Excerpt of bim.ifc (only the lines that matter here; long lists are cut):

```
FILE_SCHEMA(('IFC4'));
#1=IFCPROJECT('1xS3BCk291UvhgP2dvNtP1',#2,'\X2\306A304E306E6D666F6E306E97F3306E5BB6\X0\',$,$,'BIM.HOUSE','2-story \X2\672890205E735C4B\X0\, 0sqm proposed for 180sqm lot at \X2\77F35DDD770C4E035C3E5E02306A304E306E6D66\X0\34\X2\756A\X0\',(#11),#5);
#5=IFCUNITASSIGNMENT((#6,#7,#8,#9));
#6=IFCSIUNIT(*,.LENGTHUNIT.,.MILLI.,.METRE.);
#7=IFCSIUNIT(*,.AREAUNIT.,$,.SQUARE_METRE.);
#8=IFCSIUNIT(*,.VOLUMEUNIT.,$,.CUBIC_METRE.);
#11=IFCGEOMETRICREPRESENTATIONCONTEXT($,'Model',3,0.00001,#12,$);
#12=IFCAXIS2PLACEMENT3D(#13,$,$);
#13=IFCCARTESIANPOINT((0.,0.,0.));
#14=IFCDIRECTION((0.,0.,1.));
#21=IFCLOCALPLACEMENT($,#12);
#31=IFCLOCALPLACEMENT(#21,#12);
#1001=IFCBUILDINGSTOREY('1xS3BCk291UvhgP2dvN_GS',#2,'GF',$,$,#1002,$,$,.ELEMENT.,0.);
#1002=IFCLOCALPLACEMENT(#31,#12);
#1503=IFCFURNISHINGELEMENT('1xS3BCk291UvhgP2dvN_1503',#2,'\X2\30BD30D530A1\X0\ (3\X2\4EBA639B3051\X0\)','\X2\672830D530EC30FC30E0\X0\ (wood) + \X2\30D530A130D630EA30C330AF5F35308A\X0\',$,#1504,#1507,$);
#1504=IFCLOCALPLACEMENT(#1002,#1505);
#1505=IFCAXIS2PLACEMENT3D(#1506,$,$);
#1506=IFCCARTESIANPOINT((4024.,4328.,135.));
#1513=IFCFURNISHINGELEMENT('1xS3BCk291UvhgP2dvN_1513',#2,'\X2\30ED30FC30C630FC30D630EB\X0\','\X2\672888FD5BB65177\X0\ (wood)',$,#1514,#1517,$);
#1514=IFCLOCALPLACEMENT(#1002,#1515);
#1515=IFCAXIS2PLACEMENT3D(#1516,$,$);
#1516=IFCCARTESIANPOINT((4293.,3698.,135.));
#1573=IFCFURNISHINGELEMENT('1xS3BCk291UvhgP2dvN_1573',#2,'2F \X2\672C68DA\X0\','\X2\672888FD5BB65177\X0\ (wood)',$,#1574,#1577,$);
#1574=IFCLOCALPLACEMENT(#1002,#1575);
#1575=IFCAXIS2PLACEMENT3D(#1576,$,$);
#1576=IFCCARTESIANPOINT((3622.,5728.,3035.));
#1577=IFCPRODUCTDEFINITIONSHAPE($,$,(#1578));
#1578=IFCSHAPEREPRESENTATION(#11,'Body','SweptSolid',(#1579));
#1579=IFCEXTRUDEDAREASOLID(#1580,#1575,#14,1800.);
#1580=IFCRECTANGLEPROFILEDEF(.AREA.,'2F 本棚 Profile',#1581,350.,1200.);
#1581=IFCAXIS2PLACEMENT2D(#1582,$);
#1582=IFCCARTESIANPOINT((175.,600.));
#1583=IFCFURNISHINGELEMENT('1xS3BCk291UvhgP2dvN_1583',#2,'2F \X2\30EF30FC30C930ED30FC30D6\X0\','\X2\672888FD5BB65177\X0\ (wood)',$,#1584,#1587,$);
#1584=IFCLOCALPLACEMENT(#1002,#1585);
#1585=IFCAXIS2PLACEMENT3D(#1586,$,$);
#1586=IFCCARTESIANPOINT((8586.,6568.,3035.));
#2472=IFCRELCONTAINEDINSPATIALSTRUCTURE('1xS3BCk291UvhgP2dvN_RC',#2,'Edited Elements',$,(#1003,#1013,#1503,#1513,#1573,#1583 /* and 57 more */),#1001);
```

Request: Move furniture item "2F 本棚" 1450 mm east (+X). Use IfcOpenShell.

```python
import ifcopenshell
import ifcopenshell.api.geometry
import ifcopenshell.util.placement

model = ifcopenshell.open("bim.ifc")

item = model.by_guid("1xS3BCk291UvhgP2dvN_1573")
matrix = ifcopenshell.util.placement.get_local_placement(item.ObjectPlacement)
matrix[0, 3] += 1450.0
ifcopenshell.api.geometry.edit_object_placement(model, product=item, matrix=matrix, is_si=False)

print(ifcopenshell.util.placement.get_local_placement(item.ObjectPlacement).round(3) + 0.0)

model.write("bim-out.ifc")
```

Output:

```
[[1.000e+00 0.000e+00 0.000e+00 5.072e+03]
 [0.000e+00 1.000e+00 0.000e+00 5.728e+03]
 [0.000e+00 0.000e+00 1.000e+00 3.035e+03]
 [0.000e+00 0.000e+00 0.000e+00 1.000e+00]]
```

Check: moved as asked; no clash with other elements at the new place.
